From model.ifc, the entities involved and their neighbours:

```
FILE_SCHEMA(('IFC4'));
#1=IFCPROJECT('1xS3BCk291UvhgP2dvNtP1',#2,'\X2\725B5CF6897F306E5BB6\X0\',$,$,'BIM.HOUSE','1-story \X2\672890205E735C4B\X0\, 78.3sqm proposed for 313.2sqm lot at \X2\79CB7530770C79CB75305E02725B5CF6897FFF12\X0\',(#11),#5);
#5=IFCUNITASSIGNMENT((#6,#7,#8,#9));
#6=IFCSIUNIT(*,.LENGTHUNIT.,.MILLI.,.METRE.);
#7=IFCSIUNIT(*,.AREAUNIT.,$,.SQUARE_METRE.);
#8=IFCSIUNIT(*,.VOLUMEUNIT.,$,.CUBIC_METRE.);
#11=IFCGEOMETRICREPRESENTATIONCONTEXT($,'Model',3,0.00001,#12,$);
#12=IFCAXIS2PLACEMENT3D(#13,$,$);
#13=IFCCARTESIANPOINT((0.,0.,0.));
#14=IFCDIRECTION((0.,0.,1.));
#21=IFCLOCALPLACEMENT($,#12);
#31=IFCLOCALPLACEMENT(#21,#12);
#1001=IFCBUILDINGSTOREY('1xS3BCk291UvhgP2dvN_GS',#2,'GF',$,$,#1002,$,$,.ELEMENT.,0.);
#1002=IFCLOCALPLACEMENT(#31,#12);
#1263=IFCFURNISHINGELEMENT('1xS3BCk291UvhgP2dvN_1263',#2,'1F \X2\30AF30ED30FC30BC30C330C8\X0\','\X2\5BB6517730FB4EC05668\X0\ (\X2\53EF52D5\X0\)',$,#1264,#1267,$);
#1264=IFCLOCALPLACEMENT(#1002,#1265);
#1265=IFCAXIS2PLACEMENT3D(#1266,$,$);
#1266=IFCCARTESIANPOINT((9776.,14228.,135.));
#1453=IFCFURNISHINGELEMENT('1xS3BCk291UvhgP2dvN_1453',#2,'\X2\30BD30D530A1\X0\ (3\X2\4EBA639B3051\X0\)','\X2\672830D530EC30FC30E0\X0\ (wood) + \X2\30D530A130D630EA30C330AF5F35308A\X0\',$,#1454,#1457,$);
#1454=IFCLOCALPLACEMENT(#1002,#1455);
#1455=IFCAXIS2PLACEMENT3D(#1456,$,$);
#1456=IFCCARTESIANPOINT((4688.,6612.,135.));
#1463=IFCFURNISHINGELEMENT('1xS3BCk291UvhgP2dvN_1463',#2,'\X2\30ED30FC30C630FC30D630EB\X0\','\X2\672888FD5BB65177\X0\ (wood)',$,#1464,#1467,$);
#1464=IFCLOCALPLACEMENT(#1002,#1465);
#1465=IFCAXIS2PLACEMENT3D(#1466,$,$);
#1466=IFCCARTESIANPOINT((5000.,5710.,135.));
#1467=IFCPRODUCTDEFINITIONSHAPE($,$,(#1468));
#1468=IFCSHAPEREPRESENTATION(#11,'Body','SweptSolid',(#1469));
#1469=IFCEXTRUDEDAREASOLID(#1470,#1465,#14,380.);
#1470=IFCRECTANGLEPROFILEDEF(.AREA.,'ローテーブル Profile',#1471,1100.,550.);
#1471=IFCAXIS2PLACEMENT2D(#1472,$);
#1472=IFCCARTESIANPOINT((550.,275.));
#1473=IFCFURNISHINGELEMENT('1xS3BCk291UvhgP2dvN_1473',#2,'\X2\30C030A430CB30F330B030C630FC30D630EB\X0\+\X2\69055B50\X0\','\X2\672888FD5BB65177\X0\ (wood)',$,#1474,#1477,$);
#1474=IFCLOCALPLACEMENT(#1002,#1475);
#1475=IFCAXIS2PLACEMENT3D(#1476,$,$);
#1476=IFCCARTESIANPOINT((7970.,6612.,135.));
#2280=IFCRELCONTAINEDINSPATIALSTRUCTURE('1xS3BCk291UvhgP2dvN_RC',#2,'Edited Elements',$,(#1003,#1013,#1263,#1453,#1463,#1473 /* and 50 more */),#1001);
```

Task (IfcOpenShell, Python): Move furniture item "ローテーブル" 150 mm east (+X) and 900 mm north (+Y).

```python
import ifcopenshell
import ifcopenshell.api.geometry
import ifcopenshell.util.placement
import ifcopenshell.util.unit

model = ifcopenshell.open("model.ifc")
unit_scale = ifcopenshell.util.unit.calculate_unit_scale(model)

item = model.by_id(1463)
matrix = ifcopenshell.util.placement.get_local_placement(item.ObjectPlacement)
matrix[0, 3] += 0.15 / unit_scale
matrix[1, 3] += 0.9 / unit_scale
ifcopenshell.api.geometry.edit_object_placement(model, product=item, matrix=matrix, is_si=False)

print(ifcopenshell.util.placement.get_local_placement(item.ObjectPlacement).round(3) + 0.0)

model.write("model-out.ifc")
```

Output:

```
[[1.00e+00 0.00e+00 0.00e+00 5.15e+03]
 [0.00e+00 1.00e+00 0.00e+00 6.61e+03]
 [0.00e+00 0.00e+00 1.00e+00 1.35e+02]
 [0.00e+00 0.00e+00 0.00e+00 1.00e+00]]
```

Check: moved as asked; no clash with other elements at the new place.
